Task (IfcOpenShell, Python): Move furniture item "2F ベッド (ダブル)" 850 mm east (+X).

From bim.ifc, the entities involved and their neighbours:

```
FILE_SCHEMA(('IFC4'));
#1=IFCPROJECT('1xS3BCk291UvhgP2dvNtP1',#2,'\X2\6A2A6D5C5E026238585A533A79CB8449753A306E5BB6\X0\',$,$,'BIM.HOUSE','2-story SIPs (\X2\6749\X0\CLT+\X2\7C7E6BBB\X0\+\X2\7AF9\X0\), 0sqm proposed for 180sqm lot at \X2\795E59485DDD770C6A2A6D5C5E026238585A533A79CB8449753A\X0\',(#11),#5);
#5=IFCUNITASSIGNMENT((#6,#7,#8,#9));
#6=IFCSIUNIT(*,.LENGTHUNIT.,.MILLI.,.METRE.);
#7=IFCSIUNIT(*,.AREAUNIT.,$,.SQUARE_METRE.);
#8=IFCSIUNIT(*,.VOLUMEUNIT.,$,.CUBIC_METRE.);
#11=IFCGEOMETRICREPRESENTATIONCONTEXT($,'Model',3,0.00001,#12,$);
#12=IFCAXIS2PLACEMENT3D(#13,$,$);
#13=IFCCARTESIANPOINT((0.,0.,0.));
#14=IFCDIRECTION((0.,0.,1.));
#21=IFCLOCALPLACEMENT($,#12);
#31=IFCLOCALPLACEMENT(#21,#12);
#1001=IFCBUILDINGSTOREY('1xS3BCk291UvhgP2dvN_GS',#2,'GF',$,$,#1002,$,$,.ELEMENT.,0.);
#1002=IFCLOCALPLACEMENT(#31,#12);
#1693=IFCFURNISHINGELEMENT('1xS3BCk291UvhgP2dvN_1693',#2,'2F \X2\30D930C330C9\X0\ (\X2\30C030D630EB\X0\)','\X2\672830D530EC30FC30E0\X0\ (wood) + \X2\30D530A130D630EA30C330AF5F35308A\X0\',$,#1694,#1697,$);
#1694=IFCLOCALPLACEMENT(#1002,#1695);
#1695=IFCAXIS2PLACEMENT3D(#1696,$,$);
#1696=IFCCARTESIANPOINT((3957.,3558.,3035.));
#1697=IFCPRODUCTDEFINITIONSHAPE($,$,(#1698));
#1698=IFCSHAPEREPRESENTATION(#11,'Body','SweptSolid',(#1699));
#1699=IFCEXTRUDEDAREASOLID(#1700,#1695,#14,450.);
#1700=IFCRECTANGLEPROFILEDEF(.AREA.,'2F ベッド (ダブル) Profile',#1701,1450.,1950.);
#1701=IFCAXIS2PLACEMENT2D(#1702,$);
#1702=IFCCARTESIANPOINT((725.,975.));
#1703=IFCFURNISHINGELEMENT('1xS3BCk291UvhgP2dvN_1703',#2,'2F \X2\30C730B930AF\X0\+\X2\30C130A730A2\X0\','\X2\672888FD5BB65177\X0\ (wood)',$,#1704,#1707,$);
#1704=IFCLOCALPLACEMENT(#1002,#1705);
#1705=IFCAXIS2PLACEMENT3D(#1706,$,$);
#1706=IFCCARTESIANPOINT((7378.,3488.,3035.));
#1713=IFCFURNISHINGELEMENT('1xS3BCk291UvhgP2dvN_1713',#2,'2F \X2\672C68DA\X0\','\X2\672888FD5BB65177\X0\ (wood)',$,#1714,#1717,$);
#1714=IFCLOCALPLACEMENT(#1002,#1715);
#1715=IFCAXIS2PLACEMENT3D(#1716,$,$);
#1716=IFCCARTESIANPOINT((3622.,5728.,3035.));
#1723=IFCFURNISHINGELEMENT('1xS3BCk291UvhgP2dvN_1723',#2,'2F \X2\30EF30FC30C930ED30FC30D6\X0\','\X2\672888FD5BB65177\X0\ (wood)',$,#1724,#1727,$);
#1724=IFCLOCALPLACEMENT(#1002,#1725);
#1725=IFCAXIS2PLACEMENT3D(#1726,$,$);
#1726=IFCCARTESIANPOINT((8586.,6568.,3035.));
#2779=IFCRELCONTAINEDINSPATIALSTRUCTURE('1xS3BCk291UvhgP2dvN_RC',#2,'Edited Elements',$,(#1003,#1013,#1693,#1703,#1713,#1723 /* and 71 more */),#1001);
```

```python
import ifcopenshell
import ifcopenshell.api.geometry
import ifcopenshell.util.placement
import ifcopenshell.util.unit

model = ifcopenshell.open("bim.ifc")
unit_scale = ifcopenshell.util.unit.calculate_unit_scale(model)

item = model.by_guid("1xS3BCk291UvhgP2dvN_1693")
matrix = ifcopenshell.util.placement.get_local_placement(item.ObjectPlacement)
matrix[0, 3] += 0.85 / unit_scale
ifcopenshell.api.geometry.edit_object_placement(model, product=item, matrix=matrix, is_si=False)

print(ifcopenshell.util.placement.get_local_placement(item.ObjectPlacement).round(3) + 0.0)

model.write("bim_rev.ifc")
```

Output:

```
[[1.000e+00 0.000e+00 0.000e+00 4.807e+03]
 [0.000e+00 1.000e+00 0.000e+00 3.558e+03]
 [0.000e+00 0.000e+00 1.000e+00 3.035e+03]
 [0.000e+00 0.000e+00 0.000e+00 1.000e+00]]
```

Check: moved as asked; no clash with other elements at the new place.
